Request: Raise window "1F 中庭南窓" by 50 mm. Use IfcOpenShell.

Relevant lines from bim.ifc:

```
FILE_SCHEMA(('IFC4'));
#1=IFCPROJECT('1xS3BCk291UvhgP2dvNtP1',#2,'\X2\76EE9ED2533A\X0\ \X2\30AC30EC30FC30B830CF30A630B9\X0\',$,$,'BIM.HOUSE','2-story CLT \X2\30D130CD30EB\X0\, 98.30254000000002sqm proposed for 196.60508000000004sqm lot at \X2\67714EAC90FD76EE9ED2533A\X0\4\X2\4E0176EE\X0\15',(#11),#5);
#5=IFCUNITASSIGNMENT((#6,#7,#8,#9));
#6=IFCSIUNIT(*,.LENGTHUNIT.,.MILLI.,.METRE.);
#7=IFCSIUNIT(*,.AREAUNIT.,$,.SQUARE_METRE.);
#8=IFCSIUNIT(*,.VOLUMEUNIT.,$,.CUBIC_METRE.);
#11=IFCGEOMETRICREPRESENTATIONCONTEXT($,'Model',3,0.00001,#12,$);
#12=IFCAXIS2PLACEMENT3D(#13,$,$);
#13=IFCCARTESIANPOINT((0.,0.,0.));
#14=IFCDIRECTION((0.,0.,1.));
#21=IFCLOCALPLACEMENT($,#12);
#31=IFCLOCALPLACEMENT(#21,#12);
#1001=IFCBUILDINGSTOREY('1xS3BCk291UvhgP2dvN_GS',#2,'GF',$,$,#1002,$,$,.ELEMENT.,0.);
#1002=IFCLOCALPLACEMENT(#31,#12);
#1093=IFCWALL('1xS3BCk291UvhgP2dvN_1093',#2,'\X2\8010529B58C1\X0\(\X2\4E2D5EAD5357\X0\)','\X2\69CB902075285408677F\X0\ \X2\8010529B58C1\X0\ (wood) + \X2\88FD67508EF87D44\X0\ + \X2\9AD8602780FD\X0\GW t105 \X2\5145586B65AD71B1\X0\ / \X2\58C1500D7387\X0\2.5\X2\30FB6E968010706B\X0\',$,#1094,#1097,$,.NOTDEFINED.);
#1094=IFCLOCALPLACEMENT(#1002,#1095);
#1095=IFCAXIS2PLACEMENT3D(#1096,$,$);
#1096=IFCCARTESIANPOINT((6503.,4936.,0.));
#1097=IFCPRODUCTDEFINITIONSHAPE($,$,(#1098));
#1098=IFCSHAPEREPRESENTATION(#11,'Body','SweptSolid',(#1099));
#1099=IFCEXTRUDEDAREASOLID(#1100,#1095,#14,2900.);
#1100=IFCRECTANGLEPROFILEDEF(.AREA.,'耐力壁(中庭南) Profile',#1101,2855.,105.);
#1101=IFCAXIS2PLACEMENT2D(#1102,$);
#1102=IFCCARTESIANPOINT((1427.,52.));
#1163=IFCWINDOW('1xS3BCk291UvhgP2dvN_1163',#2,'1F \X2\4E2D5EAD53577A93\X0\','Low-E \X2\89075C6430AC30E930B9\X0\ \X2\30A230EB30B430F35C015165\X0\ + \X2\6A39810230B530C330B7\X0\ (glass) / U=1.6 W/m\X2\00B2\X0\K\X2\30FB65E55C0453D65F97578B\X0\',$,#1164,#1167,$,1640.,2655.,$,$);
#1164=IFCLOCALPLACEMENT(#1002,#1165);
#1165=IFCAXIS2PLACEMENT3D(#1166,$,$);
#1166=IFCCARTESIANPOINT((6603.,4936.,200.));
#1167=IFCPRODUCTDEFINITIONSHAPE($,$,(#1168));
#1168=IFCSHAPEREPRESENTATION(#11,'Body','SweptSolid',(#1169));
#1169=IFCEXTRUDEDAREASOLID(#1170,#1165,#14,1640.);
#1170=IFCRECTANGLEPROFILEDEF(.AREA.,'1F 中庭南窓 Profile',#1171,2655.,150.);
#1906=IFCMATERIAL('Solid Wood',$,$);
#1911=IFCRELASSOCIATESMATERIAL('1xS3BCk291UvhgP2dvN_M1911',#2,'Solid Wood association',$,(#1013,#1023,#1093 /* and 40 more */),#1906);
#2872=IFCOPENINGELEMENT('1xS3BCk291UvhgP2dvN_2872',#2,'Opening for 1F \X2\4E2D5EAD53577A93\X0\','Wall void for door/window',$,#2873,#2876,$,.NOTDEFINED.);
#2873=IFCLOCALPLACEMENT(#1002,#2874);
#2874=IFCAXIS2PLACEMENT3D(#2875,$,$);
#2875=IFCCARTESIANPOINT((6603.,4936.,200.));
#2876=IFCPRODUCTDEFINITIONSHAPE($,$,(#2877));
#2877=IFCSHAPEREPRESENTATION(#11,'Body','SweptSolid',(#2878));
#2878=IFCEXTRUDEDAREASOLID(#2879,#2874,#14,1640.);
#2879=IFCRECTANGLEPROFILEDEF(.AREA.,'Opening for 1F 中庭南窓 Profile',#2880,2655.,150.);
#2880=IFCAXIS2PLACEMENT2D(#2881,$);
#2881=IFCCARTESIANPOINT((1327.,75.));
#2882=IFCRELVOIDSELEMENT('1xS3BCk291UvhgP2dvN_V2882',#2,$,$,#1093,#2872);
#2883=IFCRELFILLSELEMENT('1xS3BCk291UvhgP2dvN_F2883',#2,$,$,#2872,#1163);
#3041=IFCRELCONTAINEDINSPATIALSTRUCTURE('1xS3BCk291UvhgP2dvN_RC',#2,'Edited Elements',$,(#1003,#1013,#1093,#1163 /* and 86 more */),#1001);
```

```python
import numpy as np
import ifcopenshell
import ifcopenshell.api.geometry
import ifcopenshell.util.placement
import ifcopenshell.util.unit

model = ifcopenshell.open("bim.ifc")
unit_scale = ifcopenshell.util.unit.calculate_unit_scale(model)

window = model.by_id(1163)
opening = window.FillsVoids[0].RelatingOpeningElement
dz = 0.05 / unit_scale

shift = np.array([0.0, 0.0, dz])
# The window is not placed relative to its opening, so move both.
for product in (opening, window):
    matrix = ifcopenshell.util.placement.get_local_placement(product.ObjectPlacement)
    matrix[:3, 3] += shift
    ifcopenshell.api.geometry.edit_object_placement(model, product=product, matrix=matrix, is_si=False)

print(f"moved by {dz * unit_scale:+.3f} m")

model.write("bim_rev.ifc")
```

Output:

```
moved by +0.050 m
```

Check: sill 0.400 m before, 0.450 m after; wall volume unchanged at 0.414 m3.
